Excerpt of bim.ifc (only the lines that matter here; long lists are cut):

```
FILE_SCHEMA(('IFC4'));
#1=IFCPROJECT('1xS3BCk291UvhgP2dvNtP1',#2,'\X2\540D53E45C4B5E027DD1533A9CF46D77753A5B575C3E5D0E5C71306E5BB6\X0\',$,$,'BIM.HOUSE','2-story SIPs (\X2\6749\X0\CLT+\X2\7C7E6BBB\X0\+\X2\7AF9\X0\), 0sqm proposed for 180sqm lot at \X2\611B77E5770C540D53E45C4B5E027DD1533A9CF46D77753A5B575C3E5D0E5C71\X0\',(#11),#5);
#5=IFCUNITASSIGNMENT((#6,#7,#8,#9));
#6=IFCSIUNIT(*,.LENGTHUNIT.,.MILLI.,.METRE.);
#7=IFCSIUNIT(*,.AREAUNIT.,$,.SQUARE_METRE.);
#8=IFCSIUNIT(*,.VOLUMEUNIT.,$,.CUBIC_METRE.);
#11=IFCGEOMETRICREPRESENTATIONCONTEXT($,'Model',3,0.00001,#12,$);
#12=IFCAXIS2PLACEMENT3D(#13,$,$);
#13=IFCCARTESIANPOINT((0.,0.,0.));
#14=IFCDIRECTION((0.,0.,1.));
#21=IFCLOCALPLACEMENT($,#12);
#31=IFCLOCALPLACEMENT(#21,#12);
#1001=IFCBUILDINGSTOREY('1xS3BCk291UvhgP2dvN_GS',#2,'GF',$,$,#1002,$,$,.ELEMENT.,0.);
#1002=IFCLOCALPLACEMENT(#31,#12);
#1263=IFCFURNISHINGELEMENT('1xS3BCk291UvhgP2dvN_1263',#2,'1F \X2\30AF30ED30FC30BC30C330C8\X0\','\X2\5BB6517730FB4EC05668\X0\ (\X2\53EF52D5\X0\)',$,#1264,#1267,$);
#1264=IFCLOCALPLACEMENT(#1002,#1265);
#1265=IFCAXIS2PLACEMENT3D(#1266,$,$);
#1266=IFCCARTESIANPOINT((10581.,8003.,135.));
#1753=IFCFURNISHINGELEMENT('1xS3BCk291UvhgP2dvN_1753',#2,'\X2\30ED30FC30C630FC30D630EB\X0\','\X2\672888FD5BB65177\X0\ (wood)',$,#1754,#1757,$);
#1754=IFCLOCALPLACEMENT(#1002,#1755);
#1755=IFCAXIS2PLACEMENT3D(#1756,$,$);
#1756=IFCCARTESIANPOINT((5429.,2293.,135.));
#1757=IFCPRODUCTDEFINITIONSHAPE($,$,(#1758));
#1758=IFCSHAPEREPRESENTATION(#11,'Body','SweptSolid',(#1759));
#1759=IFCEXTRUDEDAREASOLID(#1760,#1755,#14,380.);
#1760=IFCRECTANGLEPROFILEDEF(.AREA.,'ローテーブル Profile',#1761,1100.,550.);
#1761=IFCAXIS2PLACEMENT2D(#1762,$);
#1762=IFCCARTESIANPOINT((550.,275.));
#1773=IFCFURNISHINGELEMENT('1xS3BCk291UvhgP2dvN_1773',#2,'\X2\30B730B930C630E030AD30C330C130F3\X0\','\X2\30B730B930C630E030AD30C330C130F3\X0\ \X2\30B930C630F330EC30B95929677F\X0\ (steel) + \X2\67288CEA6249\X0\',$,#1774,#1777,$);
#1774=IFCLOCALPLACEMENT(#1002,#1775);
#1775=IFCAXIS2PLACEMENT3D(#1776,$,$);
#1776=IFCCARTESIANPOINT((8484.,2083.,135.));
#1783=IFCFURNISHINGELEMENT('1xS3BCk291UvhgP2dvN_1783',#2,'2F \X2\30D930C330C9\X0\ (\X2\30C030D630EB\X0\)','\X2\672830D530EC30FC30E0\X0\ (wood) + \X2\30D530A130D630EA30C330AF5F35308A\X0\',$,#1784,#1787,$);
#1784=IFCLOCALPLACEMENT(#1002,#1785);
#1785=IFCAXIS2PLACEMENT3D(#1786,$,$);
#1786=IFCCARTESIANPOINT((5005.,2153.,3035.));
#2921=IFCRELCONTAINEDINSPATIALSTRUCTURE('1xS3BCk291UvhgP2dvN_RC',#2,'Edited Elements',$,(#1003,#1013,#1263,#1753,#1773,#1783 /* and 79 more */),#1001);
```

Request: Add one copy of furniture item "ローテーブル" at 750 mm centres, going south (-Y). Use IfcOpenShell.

```python
import numpy as np
import ifcopenshell
import ifcopenshell.api.geometry
import ifcopenshell.api.root
import ifcopenshell.util.element
import ifcopenshell.util.placement
import ifcopenshell.util.unit

model = ifcopenshell.open("bim.ifc")
unit_scale = ifcopenshell.util.unit.calculate_unit_scale(model)


def reuse_history(source, copy):
    """copy_class also copies each property set's owner history, people and application; keep the originals."""
    for rel in copy.IsDefinedBy:
        if rel.is_a("IfcRelDefinesByProperties") and (history := rel.RelatingPropertyDefinition.OwnerHistory):
            rel.RelatingPropertyDefinition.OwnerHistory = source.OwnerHistory
            ifcopenshell.util.element.remove_deep2(model, history)


source = model.by_id(1753)
base = ifcopenshell.util.placement.get_local_placement(source.ObjectPlacement)
step = np.array([0.0, -1.0, 0.0]) * 0.75 / unit_scale

for i in range(1, 2):
    copy = ifcopenshell.api.root.copy_class(model, product=source)
    copy.Representation = ifcopenshell.util.element.copy_deep(
        model, source.Representation, exclude=["IfcGeometricRepresentationContext", "IfcRepresentationMap"]
    )
    reuse_history(source, copy)
    matrix = base.copy()
    matrix[:3, 3] += i * step
    print("added at", matrix[:3, 3].round(3) + 0.0)
    ifcopenshell.api.geometry.edit_object_placement(model, product=copy, matrix=matrix, is_si=False)

model.write("bim_edited.ifc")
```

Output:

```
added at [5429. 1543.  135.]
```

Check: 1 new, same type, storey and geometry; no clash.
